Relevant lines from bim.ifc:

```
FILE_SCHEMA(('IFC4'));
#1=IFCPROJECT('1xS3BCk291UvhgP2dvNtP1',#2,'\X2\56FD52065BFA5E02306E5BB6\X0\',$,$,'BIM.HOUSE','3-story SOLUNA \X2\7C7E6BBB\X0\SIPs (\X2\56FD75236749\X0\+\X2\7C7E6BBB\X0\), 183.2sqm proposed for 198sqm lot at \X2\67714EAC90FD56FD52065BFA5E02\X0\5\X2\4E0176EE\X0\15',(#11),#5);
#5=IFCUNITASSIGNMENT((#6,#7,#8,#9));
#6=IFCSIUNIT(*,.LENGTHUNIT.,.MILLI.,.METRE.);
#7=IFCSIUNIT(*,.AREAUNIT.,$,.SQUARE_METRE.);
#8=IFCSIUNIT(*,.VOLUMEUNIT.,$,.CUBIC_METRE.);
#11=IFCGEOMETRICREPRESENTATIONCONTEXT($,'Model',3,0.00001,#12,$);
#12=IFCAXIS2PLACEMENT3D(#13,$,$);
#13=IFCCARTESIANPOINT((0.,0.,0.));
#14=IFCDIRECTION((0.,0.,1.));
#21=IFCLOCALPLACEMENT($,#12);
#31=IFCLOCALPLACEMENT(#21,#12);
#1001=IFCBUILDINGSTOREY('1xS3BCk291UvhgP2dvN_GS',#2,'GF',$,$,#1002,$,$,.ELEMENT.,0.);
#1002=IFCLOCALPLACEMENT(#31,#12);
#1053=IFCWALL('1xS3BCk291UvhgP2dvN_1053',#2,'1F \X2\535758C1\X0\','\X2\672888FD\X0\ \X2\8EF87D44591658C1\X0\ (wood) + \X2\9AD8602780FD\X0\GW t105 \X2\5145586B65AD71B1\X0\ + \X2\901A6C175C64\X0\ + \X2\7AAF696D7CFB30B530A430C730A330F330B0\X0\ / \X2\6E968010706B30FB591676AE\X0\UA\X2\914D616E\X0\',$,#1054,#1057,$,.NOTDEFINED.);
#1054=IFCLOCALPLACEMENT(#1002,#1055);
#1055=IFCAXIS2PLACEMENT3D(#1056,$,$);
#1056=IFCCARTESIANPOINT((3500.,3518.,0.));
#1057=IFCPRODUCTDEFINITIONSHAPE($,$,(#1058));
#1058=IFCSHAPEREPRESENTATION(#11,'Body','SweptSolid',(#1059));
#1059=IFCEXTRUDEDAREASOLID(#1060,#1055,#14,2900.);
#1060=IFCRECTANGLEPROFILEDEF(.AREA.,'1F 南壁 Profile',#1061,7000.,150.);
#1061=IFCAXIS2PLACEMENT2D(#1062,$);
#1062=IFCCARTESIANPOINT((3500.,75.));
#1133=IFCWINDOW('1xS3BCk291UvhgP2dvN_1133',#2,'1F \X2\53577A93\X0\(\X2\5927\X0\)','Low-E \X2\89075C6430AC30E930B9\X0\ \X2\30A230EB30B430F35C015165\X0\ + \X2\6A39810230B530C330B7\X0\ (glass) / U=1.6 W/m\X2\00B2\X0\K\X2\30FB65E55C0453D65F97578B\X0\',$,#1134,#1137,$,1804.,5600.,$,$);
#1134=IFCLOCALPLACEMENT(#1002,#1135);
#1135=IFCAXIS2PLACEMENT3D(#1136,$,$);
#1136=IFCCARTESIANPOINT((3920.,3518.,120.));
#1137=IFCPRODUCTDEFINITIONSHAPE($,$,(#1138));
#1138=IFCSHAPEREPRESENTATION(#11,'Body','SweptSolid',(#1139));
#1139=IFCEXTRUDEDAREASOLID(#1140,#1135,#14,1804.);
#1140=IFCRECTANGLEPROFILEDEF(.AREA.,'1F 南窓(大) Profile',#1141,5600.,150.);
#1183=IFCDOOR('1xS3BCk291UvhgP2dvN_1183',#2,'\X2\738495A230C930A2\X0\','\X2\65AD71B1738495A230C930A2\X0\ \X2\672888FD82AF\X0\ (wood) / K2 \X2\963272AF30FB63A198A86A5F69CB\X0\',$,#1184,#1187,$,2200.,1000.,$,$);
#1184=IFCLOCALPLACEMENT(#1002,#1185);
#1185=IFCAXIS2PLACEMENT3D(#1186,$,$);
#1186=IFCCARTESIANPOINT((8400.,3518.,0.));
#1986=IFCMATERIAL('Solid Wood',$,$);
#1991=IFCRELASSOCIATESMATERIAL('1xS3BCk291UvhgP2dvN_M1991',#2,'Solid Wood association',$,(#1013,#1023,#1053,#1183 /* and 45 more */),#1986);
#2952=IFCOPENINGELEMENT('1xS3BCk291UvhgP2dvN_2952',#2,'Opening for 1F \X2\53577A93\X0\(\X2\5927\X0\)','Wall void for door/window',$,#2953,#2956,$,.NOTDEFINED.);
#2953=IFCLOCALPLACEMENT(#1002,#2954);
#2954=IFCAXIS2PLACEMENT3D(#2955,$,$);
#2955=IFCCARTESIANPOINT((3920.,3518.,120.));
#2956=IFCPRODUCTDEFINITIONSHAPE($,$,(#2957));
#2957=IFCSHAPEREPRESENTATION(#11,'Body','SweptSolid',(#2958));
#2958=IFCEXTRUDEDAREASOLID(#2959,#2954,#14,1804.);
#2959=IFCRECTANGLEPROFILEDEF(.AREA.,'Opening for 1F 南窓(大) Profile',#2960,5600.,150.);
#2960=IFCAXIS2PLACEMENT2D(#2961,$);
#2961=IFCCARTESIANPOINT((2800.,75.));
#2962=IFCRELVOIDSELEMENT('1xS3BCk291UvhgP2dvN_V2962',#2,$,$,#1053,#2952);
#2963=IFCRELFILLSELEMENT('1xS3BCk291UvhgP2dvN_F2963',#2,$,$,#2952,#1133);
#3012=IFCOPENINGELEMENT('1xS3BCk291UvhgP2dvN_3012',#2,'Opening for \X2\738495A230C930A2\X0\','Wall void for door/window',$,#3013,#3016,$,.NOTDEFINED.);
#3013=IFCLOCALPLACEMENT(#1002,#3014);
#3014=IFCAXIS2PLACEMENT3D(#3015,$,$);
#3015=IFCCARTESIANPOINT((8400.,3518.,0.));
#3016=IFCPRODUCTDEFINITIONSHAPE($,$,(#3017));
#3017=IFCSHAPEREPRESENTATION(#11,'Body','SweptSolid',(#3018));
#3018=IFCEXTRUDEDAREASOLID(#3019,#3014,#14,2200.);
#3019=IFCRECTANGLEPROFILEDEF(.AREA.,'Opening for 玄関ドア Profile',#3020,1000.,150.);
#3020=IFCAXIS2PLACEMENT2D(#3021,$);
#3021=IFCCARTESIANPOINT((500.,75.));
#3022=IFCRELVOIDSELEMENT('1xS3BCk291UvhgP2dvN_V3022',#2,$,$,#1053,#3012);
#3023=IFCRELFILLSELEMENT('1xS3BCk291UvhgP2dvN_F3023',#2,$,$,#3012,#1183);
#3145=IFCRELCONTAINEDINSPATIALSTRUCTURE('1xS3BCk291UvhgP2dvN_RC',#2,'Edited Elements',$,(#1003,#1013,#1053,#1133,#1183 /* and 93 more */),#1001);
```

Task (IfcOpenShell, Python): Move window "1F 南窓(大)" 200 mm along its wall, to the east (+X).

```python
import ifcopenshell
import ifcopenshell.api.geometry
import ifcopenshell.util.placement

model = ifcopenshell.open("bim.ifc")

window = model.by_guid("1xS3BCk291UvhgP2dvN_1133")
opening = window.FillsVoids[0].RelatingOpeningElement
wall = opening.VoidsElements[0].RelatingBuildingElement

wall_matrix = ifcopenshell.util.placement.get_local_placement(wall.ObjectPlacement)
shift = wall_matrix[:3, 0] * 200.0
before = ifcopenshell.util.placement.get_local_placement(window.ObjectPlacement)[:3, 3].copy()

# The window is not placed relative to its opening, so move both.
for product in (opening, window):
    matrix = ifcopenshell.util.placement.get_local_placement(product.ObjectPlacement)
    matrix[:3, 3] += shift
    ifcopenshell.api.geometry.edit_object_placement(model, product=product, matrix=matrix, is_si=False)

after = ifcopenshell.util.placement.get_local_placement(window.ObjectPlacement)[:3, 3]
print("window moved by", (after - before).round(3) + 0.0)

model.write("bim_v2.ifc")
```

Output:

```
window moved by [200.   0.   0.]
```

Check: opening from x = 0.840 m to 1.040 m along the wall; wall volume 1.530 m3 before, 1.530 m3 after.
